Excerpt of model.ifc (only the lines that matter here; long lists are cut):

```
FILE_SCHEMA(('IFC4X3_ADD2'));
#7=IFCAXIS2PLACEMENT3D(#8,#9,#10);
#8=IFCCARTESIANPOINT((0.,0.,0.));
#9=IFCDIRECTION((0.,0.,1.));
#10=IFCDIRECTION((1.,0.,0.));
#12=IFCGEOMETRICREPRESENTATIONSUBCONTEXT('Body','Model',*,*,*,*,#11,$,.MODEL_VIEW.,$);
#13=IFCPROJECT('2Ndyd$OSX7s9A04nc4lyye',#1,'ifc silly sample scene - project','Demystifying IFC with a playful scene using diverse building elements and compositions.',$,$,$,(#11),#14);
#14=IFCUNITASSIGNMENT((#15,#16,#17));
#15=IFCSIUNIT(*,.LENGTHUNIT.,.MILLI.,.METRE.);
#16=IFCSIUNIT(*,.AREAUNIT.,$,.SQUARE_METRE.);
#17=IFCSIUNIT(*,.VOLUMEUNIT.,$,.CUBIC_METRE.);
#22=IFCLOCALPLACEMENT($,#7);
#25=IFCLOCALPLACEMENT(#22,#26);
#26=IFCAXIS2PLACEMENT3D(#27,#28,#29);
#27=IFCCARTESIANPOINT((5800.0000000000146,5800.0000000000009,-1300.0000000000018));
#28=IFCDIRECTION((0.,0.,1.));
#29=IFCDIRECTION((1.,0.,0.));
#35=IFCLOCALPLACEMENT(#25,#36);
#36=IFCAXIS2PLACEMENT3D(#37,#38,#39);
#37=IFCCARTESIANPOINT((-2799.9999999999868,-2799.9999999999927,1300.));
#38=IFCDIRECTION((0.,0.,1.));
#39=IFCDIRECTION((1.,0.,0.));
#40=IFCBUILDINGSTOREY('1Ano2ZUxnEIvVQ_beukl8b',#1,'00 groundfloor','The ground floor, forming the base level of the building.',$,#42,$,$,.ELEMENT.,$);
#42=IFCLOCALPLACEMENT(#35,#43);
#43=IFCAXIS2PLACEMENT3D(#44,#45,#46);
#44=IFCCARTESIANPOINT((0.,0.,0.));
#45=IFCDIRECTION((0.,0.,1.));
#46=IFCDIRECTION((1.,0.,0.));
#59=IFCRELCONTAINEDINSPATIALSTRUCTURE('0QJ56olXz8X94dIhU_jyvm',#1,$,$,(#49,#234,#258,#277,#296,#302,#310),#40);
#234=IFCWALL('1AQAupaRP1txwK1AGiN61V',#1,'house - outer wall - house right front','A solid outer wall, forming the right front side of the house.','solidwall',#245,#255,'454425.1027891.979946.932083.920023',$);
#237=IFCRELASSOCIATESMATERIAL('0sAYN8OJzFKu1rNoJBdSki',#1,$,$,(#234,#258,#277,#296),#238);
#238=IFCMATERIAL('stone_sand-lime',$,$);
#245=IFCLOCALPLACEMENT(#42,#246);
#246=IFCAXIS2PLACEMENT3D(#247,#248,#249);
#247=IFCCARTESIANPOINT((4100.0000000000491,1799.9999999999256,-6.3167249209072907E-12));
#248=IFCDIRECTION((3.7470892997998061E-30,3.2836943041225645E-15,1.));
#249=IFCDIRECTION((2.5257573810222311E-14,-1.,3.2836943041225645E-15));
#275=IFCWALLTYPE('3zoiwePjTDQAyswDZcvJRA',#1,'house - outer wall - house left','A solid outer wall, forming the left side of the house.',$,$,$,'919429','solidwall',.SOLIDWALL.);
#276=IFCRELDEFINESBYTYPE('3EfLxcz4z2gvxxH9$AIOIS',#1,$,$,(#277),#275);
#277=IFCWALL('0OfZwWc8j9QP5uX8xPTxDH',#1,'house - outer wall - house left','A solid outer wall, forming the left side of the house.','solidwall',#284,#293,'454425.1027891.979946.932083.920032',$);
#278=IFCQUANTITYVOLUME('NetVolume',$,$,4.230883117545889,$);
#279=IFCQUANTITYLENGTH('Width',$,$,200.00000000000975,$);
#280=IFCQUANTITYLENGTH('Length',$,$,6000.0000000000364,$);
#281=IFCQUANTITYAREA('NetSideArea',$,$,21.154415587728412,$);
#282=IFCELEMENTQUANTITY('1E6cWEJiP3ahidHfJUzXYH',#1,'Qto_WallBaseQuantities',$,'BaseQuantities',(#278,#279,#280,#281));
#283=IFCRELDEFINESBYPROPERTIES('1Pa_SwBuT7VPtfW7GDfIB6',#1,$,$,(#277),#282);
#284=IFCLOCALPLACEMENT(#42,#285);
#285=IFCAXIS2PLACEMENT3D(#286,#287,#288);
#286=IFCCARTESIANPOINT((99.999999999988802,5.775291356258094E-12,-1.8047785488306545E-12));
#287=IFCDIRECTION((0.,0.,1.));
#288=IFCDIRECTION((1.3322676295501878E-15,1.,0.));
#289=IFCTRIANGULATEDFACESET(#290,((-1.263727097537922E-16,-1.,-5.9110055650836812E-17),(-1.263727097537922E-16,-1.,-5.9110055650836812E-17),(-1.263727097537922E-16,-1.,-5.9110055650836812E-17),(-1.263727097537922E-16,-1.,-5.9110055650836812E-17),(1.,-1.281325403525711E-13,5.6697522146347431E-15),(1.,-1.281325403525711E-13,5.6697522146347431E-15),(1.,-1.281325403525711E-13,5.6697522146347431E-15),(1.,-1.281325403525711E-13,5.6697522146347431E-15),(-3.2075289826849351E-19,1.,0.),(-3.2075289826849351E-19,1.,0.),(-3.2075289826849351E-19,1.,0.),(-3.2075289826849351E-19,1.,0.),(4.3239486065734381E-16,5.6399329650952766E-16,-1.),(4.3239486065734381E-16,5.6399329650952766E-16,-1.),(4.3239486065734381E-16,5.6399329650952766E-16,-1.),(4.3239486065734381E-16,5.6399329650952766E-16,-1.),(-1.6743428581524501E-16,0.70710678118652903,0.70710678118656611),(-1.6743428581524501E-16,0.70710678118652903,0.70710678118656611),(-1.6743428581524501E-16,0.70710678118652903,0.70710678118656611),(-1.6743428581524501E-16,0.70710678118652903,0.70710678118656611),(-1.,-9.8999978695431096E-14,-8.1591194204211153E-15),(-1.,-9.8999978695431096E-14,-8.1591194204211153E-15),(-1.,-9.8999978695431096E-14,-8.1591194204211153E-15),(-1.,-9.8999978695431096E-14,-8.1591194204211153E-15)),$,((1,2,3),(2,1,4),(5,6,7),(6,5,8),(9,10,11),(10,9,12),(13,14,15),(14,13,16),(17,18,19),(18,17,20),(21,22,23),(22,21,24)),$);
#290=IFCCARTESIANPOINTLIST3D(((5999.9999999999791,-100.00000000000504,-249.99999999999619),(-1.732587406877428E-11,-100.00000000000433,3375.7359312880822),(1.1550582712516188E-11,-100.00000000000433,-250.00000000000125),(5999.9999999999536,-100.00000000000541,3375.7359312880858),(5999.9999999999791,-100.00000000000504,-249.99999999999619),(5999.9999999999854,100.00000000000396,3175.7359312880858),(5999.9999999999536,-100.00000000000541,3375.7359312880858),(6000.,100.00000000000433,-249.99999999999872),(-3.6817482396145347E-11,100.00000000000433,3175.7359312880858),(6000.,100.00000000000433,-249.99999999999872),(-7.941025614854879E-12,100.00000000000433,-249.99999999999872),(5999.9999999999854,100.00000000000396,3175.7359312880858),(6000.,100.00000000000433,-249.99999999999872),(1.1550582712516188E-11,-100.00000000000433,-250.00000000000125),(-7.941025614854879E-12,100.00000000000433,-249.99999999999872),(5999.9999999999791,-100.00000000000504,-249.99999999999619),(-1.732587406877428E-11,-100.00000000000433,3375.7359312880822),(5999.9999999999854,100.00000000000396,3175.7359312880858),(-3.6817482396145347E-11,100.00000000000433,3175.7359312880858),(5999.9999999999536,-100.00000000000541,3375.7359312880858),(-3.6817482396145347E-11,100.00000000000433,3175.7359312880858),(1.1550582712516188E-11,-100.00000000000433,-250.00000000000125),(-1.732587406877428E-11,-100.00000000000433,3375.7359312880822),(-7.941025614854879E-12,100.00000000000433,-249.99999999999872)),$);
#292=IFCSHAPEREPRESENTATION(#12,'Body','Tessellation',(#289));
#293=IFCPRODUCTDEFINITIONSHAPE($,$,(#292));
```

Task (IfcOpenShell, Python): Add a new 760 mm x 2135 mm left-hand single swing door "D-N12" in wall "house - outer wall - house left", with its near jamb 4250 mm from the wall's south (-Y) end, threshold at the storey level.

```python
import numpy as np
import ifcopenshell
import ifcopenshell.api.feature
import ifcopenshell.api.geometry
import ifcopenshell.api.pset
import ifcopenshell.api.root
import ifcopenshell.api.spatial
import ifcopenshell.geom
import ifcopenshell.util.element
import ifcopenshell.util.placement
import ifcopenshell.util.representation
import ifcopenshell.util.shape
import ifcopenshell.util.unit

model = ifcopenshell.open("model.ifc")
unit_scale = ifcopenshell.util.unit.calculate_unit_scale(model)
area_scale = ifcopenshell.util.unit.calculate_unit_scale(model, "AREAUNIT")
volume_scale = ifcopenshell.util.unit.calculate_unit_scale(model, "VOLUMEUNIT")
settings = ifcopenshell.geom.settings()


def volume(element):
    """Net volume in cubic metres, openings subtracted."""
    shape = ifcopenshell.geom.create_shape(settings, element)
    return ifcopenshell.util.shape.get_volume(shape.geometry)


wall = model.by_guid("0OfZwWc8j9QP5uX8xPTxDH")
storey = ifcopenshell.util.element.get_container(wall, ifc_class="IfcBuildingStorey")
context = ifcopenshell.util.representation.get_context(model, "Model", "Body", "MODEL_VIEW")
before = volume(wall)

width, height, from_end, sill = 0.76, 2.135, 4.25, 0.0  # metres

# The wall runs along its own X axis, and the end named is its -X end.
wall_shape = ifcopenshell.geom.create_shape(settings, wall)
x, y, z = ifcopenshell.util.shape.get_vertices(wall_shape.geometry).T
start = x.min() + from_end
face, thickness = float(y.min()), float(y.max() - y.min())
wall_matrix = ifcopenshell.util.placement.get_local_placement(wall.ObjectPlacement)
level = ifcopenshell.util.placement.get_local_placement(storey.ObjectPlacement)[2, 3]


def in_wall(x, y):
    """Placement at x, y metres in the wall's axes, at sill height."""
    matrix = wall_matrix.copy()
    matrix[:, 3] = wall_matrix @ np.array([x / unit_scale, y / unit_scale, 0.0, 1.0])
    matrix[2, 3] = level + sill / unit_scale
    return matrix


# Opening: a box that overshoots both wall faces by 50 mm.
opening = ifcopenshell.api.root.create_entity(model, ifc_class="IfcOpeningElement", predefined_type="OPENING")
box = ifcopenshell.api.geometry.add_wall_representation(
    model, context=context, length=width, height=height, thickness=thickness + 0.1
)
ifcopenshell.api.geometry.assign_representation(model, product=opening, representation=box)
ifcopenshell.api.geometry.edit_object_placement(model, product=opening, matrix=in_wall(start, face - 0.05), is_si=False)
ifcopenshell.api.feature.add_feature(model, feature=opening, element=wall)

door = ifcopenshell.api.root.create_entity(model, ifc_class="IfcDoor", name="D-N12", predefined_type="DOOR")
door.OverallWidth, door.OverallHeight = width / unit_scale, height / unit_scale
door.OperationType = "SINGLE_SWING_LEFT"
body = ifcopenshell.api.geometry.add_door_representation(
    model,
    context=context,
    overall_width=door.OverallWidth,
    overall_height=door.OverallHeight,
    operation_type="SINGLE_SWING_LEFT",
    lining_properties={"LiningDepth": thickness / unit_scale, "ThresholdDepth": thickness / unit_scale},
)
ifcopenshell.api.geometry.assign_representation(model, product=door, representation=body)
ifcopenshell.api.spatial.assign_container(model, products=[door], relating_structure=storey)
ifcopenshell.api.feature.add_filling(model, opening=opening, element=door)

# The lining spans the wall, so the door starts at the wall face.
ifcopenshell.api.geometry.edit_object_placement(model, product=door, matrix=in_wall(start, face), is_si=False)

after = volume(wall)

# Update the wall's stored quantities.
qto = model.by_id(ifcopenshell.util.element.get_pset(wall, "Qto_WallBaseQuantities", should_inherit=False)["id"])
ifcopenshell.api.pset.edit_qto(model, qto=qto, properties={
    "NetVolume": after / volume_scale,
    "NetSideArea": after / thickness / area_scale,
})

print(f"wall volume {before:.3f} -> {after:.3f} m3")

model.write("model_edited.ifc")
```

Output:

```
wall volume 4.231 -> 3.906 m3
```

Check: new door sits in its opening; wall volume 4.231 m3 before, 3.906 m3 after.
